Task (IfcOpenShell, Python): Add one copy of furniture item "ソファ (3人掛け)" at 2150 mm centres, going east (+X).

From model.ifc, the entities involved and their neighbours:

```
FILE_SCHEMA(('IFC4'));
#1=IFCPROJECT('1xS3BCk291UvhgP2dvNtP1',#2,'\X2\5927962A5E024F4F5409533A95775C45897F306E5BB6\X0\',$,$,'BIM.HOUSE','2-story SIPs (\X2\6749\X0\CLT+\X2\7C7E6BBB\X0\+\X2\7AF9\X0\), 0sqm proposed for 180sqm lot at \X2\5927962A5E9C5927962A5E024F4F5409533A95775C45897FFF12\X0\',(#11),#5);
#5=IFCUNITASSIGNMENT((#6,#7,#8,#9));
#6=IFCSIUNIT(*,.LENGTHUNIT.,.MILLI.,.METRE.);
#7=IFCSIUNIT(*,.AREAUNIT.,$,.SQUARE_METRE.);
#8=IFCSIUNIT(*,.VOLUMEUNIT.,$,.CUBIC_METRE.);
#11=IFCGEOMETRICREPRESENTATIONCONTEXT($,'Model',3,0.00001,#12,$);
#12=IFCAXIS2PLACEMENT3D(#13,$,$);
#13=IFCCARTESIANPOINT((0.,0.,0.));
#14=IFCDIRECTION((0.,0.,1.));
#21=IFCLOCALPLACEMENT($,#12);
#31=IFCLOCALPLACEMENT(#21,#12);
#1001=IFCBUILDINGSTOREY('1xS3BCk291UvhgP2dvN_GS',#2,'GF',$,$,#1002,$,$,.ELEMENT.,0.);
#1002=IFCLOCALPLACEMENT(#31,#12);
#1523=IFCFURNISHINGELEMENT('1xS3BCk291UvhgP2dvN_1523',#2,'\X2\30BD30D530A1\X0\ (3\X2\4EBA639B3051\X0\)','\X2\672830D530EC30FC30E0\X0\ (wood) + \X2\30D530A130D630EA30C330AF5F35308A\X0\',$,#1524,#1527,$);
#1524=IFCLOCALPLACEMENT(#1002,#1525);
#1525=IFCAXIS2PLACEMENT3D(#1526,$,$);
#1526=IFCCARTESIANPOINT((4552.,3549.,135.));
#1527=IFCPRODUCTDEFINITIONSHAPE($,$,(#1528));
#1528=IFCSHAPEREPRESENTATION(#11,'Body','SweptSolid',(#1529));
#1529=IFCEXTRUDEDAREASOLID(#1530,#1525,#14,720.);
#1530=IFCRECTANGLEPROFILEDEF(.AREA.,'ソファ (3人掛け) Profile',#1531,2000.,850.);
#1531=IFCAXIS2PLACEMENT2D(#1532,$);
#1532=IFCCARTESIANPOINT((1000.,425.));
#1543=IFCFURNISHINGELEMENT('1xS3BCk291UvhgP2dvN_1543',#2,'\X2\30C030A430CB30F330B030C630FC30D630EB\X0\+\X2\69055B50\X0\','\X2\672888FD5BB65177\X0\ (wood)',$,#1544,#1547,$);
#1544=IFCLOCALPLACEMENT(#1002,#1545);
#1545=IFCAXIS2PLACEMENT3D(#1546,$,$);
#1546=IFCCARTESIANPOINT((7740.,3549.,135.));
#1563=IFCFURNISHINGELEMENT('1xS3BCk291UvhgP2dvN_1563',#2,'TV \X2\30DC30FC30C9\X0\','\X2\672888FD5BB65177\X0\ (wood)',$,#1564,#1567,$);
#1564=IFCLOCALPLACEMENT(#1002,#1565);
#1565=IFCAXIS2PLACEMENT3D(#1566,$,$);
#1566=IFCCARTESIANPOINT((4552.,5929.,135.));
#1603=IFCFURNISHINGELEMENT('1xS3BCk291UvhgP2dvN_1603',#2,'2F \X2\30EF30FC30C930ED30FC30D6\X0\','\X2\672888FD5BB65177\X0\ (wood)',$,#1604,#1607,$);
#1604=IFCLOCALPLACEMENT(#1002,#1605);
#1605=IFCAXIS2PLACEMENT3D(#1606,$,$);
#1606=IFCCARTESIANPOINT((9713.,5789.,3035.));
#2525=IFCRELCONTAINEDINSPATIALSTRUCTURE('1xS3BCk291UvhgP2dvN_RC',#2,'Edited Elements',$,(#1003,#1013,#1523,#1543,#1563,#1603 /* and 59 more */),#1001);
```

```python
import numpy as np
import ifcopenshell
import ifcopenshell.api.geometry
import ifcopenshell.api.root
import ifcopenshell.util.element
import ifcopenshell.util.placement

model = ifcopenshell.open("model.ifc")


def reuse_history(source, copy):
    """copy_class also copies each property set's owner history, people and application; keep the originals."""
    for rel in copy.IsDefinedBy:
        if rel.is_a("IfcRelDefinesByProperties") and (history := rel.RelatingPropertyDefinition.OwnerHistory):
            rel.RelatingPropertyDefinition.OwnerHistory = source.OwnerHistory
            ifcopenshell.util.element.remove_deep2(model, history)


source = model.by_guid("1xS3BCk291UvhgP2dvN_1523")
base = ifcopenshell.util.placement.get_local_placement(source.ObjectPlacement)
step = np.array([1.0, 0.0, 0.0]) * 2150.0

for i in range(1, 2):
    copy = ifcopenshell.api.root.copy_class(model, product=source)
    copy.Representation = ifcopenshell.util.element.copy_deep(
        model, source.Representation, exclude=["IfcGeometricRepresentationContext", "IfcRepresentationMap"]
    )
    reuse_history(source, copy)
    matrix = base.copy()
    matrix[:3, 3] += i * step
    print("added at", matrix[:3, 3].round(3) + 0.0)
    ifcopenshell.api.geometry.edit_object_placement(model, product=copy, matrix=matrix, is_si=False)

model.write("model_edited.ifc")
```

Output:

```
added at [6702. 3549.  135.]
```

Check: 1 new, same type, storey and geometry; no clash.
